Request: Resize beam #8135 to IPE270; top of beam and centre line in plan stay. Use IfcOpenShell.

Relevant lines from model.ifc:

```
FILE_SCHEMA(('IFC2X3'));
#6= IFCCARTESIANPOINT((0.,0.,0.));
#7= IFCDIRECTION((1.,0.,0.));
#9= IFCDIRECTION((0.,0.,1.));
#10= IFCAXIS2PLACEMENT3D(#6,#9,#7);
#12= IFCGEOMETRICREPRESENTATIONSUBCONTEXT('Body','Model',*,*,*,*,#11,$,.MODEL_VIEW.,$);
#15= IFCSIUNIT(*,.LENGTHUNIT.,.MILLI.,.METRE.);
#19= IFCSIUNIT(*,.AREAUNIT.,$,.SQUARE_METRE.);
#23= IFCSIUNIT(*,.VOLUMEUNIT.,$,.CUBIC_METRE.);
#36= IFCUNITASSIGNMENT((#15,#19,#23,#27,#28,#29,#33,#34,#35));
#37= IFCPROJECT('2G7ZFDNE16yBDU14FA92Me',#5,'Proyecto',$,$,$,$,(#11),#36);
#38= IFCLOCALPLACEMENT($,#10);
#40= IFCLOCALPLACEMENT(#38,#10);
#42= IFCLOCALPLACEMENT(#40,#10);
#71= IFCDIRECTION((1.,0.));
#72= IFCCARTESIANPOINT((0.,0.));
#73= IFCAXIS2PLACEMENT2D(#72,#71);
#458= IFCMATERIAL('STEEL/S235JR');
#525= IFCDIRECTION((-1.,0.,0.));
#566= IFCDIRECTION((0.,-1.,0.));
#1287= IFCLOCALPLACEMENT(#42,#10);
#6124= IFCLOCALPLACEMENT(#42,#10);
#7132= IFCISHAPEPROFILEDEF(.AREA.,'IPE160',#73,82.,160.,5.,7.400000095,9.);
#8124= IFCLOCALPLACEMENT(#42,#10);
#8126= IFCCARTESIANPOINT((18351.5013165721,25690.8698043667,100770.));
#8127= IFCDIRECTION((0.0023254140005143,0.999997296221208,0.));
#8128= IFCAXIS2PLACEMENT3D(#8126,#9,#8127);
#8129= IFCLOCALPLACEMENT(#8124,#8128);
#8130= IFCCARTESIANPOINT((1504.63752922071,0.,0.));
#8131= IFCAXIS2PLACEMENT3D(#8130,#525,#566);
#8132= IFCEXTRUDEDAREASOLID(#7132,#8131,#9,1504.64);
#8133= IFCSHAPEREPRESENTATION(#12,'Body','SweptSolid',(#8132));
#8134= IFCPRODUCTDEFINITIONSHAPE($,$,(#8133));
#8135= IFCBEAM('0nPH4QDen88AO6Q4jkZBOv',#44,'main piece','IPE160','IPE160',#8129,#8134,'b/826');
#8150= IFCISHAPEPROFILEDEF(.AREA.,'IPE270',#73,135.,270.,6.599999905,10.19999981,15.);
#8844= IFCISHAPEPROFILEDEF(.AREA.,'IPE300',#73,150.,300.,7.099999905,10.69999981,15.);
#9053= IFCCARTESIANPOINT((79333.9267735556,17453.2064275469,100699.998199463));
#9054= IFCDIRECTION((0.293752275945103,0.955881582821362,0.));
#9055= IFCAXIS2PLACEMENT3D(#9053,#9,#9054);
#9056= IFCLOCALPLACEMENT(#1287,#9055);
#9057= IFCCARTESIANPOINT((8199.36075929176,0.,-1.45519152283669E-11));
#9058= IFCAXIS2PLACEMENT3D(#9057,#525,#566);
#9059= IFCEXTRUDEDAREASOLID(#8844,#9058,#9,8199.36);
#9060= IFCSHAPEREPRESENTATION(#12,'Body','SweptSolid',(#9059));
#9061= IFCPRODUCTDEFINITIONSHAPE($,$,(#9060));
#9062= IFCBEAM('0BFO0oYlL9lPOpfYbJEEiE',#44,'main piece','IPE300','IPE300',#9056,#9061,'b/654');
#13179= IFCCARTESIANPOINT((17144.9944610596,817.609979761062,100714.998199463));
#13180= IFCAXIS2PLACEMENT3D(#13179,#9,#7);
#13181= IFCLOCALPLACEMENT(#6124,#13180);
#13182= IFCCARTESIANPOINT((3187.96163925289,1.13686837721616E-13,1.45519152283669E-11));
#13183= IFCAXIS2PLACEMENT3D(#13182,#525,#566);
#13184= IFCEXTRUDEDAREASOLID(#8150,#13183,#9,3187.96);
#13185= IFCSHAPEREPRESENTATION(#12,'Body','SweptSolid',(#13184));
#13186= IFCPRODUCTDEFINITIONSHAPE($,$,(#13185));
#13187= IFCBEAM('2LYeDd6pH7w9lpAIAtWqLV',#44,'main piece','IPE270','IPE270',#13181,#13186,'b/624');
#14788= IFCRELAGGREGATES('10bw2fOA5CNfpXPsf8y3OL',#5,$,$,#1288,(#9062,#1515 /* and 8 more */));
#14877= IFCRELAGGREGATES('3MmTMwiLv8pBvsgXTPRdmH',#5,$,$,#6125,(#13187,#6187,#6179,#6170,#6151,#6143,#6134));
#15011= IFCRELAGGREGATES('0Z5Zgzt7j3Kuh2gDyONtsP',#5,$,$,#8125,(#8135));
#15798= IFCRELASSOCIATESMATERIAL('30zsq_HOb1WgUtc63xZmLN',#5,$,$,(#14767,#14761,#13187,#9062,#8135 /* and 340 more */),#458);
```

```python
import ifcopenshell
import ifcopenshell.util.element
import ifcopenshell.util.representation

model = ifcopenshell.open("model.ifc")

member = model.by_guid("0nPH4QDen88AO6Q4jkZBOv")
source = next(p for p in model.by_type("IfcIShapeProfileDef") if p.ProfileName == "IPE270")

body = ifcopenshell.util.representation.get_representation(member, "Model", "Body")
solid = body.Items[0]
old_profile = solid.SweptArea

# Copy the section's sizes but keep this member's own profile position.
profile = ifcopenshell.util.element.copy(model, source)
# Profiles are centred, so shift by half the change in depth to hold the top.
shift = (old_profile.OverallDepth - profile.OverallDepth) / 2
x, y = old_profile.Position.Location.Coordinates
up = (0.0, 1.0)  # upwards, in the solid's own plane
location = model.createIfcCartesianPoint((x + up[0] * shift, y + up[1] * shift))
profile.Position = model.createIfcAxis2Placement2D(location, old_profile.Position.RefDirection)
solid.SweptArea = profile
if not model.get_total_inverses(old_profile):
    ifcopenshell.util.element.remove_deep2(model, old_profile)
member.Description = member.Description.replace("IPE160", "IPE270")
member.ObjectType = member.ObjectType.replace("IPE160", "IPE270")

print(solid.SweptArea)

model.write("model_rev.ifc")
```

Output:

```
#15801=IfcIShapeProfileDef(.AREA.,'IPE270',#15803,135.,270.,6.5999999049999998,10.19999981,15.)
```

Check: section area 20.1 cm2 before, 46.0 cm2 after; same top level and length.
